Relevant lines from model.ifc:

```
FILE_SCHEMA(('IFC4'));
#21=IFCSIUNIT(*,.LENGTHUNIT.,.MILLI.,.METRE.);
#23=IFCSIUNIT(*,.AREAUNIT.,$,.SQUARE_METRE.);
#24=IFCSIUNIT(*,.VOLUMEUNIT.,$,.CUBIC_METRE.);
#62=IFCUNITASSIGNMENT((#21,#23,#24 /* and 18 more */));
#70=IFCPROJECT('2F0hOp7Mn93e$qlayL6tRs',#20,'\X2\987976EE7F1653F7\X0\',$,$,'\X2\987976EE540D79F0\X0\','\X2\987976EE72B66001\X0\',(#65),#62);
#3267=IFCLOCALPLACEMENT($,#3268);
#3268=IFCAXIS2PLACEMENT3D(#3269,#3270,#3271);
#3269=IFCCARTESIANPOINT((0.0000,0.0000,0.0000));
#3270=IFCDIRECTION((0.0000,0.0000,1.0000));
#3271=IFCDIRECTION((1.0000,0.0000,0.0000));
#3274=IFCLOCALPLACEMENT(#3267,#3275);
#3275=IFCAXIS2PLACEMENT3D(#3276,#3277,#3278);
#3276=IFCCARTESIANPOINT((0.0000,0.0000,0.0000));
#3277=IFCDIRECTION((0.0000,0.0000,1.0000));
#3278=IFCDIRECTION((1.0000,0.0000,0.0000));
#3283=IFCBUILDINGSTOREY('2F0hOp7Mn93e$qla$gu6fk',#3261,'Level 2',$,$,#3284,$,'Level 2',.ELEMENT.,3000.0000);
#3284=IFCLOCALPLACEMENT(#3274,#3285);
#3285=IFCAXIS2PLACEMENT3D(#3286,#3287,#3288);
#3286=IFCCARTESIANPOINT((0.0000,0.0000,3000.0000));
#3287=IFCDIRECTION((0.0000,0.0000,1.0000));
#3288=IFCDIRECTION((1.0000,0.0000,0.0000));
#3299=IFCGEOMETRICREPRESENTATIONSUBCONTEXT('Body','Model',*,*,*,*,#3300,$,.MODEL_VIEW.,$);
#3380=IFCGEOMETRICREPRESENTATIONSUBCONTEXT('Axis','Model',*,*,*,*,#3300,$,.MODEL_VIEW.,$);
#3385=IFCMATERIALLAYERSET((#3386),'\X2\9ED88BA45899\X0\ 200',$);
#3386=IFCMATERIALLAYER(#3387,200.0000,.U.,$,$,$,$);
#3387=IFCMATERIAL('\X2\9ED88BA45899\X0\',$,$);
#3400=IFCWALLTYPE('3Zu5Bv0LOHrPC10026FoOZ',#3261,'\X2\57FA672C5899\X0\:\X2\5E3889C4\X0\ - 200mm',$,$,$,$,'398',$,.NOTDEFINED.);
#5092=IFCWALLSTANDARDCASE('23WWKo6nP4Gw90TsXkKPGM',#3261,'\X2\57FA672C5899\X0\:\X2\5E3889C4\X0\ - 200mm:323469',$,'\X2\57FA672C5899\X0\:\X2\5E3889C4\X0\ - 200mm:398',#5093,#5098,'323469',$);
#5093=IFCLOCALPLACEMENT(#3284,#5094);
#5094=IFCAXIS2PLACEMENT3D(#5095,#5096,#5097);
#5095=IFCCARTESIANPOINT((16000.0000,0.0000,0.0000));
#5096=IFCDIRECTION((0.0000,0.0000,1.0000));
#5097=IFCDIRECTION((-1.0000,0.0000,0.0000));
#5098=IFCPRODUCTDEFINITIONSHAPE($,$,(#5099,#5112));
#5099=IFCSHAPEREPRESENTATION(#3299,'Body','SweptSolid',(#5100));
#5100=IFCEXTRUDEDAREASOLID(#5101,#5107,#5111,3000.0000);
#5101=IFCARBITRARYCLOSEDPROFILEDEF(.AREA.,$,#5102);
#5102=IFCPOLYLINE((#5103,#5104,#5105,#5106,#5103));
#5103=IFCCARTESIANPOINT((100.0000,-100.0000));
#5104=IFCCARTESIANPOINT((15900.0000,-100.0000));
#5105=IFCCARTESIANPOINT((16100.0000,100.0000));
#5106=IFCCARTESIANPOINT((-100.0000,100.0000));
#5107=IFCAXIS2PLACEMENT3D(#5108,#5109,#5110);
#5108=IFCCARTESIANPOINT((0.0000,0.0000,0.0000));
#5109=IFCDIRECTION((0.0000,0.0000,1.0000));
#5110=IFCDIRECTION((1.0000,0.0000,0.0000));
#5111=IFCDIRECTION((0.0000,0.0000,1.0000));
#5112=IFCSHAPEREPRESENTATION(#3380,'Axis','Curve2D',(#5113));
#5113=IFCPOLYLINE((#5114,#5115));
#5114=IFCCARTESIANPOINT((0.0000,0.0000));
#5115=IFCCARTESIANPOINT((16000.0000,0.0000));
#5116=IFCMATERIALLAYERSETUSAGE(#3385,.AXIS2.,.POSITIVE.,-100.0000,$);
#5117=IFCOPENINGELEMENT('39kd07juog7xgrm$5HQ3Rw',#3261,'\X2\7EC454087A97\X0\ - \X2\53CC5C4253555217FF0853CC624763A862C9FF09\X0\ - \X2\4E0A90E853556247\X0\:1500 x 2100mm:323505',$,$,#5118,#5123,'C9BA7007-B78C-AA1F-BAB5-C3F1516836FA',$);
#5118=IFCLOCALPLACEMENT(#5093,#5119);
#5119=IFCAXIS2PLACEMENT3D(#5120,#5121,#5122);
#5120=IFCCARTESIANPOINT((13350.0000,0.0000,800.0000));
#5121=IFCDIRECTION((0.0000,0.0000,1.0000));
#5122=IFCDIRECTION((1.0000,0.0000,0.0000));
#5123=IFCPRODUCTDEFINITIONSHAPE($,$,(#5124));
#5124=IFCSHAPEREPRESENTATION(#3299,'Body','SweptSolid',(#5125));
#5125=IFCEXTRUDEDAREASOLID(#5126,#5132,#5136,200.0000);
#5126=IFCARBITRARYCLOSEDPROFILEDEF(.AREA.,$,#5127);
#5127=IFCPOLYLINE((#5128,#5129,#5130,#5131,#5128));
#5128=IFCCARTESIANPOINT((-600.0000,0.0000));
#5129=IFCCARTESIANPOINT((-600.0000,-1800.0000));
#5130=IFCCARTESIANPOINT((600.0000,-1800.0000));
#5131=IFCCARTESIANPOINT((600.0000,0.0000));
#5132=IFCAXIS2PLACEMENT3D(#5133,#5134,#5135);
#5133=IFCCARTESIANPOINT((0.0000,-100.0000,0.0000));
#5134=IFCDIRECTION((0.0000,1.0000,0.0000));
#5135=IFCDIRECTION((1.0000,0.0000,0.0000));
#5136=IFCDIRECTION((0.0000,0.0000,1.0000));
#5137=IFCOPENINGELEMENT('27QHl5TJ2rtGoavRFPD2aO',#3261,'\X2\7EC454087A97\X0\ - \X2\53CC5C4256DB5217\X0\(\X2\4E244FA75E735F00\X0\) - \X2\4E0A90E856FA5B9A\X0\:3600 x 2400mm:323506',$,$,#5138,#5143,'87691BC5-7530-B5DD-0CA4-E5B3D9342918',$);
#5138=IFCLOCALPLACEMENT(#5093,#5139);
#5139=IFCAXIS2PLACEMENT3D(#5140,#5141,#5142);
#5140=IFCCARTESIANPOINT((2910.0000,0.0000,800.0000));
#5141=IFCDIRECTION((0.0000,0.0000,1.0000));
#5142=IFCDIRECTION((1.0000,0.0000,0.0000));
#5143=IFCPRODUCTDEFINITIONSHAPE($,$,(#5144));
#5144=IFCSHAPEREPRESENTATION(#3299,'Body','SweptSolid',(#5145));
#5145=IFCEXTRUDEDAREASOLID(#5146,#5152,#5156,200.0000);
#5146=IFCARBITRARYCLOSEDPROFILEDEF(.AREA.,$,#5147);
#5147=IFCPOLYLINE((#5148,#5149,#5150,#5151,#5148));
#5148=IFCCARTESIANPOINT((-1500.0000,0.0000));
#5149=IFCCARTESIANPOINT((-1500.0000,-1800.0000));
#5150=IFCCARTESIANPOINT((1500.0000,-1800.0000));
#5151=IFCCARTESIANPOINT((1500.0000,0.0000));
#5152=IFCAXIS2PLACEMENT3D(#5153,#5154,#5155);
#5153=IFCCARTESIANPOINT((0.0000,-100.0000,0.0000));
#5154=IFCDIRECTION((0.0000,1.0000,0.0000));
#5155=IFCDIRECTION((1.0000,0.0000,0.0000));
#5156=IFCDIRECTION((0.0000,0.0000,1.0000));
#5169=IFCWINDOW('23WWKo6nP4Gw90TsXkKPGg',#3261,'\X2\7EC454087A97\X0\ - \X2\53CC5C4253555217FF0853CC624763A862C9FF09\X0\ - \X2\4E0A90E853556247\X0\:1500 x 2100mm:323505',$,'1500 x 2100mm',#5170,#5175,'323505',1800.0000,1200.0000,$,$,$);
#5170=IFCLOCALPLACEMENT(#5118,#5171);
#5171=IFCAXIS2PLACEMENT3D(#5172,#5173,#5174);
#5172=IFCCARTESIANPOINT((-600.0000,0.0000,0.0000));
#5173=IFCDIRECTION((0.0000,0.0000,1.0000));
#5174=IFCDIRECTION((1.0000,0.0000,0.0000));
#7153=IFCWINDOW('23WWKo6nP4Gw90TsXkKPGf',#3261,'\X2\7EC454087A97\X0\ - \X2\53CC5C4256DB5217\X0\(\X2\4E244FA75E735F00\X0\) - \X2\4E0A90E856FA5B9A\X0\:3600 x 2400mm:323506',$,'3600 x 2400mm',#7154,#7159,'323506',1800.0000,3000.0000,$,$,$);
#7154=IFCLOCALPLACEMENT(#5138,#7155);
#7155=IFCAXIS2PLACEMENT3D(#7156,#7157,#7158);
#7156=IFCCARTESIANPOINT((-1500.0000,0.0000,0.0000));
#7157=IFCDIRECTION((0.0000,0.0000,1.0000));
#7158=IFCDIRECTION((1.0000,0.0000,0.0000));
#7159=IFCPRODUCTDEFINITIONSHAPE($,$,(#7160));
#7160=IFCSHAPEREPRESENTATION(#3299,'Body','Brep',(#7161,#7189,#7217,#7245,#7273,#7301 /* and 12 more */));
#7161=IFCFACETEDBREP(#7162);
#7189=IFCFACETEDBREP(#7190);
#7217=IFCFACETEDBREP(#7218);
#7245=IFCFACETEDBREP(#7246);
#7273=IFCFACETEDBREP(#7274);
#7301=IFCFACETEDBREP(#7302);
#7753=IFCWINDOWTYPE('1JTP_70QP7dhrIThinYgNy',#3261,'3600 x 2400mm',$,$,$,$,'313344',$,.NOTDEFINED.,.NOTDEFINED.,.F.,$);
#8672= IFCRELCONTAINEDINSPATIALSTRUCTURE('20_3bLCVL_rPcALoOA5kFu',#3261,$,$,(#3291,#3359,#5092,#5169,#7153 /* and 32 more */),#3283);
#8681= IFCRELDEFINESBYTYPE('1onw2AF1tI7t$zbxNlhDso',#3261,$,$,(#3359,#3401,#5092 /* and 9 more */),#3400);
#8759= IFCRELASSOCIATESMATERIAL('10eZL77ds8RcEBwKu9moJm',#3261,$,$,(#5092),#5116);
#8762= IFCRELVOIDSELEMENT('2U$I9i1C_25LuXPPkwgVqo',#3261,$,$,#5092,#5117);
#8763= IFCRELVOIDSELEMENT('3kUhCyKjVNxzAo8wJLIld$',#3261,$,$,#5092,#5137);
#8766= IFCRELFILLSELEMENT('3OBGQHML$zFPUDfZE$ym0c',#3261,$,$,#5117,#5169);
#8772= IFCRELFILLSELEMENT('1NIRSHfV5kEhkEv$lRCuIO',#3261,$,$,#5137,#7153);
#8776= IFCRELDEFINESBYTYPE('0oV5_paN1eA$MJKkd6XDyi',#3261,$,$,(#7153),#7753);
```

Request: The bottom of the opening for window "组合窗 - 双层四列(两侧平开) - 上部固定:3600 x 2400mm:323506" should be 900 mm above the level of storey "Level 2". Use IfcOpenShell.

```python
import numpy as np
import ifcopenshell
import ifcopenshell.api.geometry
import ifcopenshell.geom
import ifcopenshell.util.element
import ifcopenshell.util.placement
import ifcopenshell.util.shape
import ifcopenshell.util.unit

model = ifcopenshell.open("model.ifc")
unit_scale = ifcopenshell.util.unit.calculate_unit_scale(model)

window = model.by_id(7153)
opening = window.FillsVoids[0].RelatingOpeningElement
storey = ifcopenshell.util.element.get_container(window, ifc_class="IfcBuildingStorey")
level = ifcopenshell.util.placement.get_local_placement(storey.ObjectPlacement)[2, 3]

# The opening's origin need not be at the sill, so measure its lowest point.
shape = ifcopenshell.geom.create_shape(ifcopenshell.geom.settings(), opening)
bottom = ifcopenshell.util.shape.get_shape_bottom_elevation(shape, shape.geometry) / unit_scale
dz = level + 0.9 / unit_scale - bottom

shift = np.array([0.0, 0.0, dz])
# The window is placed relative to its opening, so it follows when the opening moves.
matrix = ifcopenshell.util.placement.get_local_placement(opening.ObjectPlacement)
matrix[:3, 3] += shift
ifcopenshell.api.geometry.edit_object_placement(
    model, product=opening, matrix=matrix, is_si=False, should_transform_children=True
)

print(f"moved by {dz * unit_scale:+.3f} m")

model.write("model-out.ifc")
```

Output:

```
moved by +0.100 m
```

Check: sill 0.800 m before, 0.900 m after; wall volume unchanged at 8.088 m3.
